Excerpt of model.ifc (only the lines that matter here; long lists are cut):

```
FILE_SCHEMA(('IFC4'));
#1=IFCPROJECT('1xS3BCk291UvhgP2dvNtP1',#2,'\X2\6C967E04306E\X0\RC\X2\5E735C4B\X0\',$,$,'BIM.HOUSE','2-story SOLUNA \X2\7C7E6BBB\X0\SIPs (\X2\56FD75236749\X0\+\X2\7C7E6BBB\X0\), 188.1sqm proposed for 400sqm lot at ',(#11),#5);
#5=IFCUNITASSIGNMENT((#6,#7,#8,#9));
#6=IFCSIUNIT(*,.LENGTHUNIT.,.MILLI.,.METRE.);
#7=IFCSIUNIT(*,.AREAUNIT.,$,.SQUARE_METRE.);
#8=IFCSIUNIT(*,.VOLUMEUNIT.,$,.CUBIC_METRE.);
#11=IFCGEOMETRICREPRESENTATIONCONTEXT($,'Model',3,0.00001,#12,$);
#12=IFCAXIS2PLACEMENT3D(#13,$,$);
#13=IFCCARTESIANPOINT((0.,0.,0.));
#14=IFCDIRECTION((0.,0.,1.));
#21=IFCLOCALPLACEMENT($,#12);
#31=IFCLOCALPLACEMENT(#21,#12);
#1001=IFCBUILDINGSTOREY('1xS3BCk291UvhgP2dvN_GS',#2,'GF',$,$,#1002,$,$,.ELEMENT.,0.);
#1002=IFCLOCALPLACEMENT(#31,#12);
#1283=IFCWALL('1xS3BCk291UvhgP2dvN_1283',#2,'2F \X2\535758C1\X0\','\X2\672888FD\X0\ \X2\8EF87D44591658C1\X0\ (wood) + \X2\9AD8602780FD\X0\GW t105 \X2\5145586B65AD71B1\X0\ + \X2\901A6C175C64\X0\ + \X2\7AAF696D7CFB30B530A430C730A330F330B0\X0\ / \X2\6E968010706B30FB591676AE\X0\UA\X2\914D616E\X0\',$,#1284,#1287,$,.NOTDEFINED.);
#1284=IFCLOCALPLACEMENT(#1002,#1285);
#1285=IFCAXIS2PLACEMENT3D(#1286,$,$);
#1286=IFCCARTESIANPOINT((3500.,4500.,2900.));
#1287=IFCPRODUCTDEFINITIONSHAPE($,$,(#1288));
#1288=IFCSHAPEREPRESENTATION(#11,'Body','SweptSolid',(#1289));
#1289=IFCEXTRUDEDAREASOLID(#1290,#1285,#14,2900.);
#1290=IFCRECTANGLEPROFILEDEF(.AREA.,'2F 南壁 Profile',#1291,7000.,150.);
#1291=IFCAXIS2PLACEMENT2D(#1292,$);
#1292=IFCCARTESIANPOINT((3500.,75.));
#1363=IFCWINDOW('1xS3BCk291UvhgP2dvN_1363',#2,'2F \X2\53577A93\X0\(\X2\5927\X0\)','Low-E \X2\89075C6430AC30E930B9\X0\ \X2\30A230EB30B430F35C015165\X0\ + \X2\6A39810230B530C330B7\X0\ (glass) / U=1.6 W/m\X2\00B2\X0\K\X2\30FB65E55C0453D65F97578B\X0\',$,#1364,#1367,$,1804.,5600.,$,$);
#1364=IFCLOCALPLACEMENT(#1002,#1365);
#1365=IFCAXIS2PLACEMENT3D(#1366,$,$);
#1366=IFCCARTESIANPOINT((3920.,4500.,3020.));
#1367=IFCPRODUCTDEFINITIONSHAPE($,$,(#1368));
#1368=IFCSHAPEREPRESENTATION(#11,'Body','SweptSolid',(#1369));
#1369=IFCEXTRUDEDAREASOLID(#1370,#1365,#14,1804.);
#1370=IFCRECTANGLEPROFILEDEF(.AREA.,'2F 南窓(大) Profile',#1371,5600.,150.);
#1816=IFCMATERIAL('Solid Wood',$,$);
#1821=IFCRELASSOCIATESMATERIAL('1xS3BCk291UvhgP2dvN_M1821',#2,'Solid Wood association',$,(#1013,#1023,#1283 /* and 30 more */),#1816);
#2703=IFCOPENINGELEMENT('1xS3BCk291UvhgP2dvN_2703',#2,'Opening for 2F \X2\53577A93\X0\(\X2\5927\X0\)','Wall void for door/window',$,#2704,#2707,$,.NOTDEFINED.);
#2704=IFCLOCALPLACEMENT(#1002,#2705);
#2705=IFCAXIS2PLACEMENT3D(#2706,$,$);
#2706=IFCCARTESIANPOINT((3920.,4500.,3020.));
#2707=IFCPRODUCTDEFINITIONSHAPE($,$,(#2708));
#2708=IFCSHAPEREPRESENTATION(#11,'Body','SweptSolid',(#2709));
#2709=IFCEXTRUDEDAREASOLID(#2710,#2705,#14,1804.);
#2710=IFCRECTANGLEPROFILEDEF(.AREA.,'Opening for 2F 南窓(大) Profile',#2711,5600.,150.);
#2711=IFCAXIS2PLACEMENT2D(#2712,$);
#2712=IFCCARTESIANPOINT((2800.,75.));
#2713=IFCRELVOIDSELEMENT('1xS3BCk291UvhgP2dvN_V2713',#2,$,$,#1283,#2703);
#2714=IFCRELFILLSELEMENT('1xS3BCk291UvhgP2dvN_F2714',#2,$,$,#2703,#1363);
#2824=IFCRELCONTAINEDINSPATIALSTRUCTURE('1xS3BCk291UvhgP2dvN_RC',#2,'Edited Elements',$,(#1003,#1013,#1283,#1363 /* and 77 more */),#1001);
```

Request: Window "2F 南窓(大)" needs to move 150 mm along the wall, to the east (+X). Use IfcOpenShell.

```python
import ifcopenshell
import ifcopenshell.api.geometry
import ifcopenshell.util.placement
import ifcopenshell.util.unit

model = ifcopenshell.open("model.ifc")
unit_scale = ifcopenshell.util.unit.calculate_unit_scale(model)

window = model.by_guid("1xS3BCk291UvhgP2dvN_1363")
opening = window.FillsVoids[0].RelatingOpeningElement
wall = opening.VoidsElements[0].RelatingBuildingElement

wall_matrix = ifcopenshell.util.placement.get_local_placement(wall.ObjectPlacement)
shift = wall_matrix[:3, 0] * 0.15 / unit_scale
before = ifcopenshell.util.placement.get_local_placement(window.ObjectPlacement)[:3, 3].copy()

# The window is not placed relative to its opening, so move both.
for product in (opening, window):
    matrix = ifcopenshell.util.placement.get_local_placement(product.ObjectPlacement)
    matrix[:3, 3] += shift
    ifcopenshell.api.geometry.edit_object_placement(model, product=product, matrix=matrix, is_si=False)

after = ifcopenshell.util.placement.get_local_placement(window.ObjectPlacement)[:3, 3]
print("window moved by", (after - before).round(3) + 0.0)

model.write("model_v2.ifc")
```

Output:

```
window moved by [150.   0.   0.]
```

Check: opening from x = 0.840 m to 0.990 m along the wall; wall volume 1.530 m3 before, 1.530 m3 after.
